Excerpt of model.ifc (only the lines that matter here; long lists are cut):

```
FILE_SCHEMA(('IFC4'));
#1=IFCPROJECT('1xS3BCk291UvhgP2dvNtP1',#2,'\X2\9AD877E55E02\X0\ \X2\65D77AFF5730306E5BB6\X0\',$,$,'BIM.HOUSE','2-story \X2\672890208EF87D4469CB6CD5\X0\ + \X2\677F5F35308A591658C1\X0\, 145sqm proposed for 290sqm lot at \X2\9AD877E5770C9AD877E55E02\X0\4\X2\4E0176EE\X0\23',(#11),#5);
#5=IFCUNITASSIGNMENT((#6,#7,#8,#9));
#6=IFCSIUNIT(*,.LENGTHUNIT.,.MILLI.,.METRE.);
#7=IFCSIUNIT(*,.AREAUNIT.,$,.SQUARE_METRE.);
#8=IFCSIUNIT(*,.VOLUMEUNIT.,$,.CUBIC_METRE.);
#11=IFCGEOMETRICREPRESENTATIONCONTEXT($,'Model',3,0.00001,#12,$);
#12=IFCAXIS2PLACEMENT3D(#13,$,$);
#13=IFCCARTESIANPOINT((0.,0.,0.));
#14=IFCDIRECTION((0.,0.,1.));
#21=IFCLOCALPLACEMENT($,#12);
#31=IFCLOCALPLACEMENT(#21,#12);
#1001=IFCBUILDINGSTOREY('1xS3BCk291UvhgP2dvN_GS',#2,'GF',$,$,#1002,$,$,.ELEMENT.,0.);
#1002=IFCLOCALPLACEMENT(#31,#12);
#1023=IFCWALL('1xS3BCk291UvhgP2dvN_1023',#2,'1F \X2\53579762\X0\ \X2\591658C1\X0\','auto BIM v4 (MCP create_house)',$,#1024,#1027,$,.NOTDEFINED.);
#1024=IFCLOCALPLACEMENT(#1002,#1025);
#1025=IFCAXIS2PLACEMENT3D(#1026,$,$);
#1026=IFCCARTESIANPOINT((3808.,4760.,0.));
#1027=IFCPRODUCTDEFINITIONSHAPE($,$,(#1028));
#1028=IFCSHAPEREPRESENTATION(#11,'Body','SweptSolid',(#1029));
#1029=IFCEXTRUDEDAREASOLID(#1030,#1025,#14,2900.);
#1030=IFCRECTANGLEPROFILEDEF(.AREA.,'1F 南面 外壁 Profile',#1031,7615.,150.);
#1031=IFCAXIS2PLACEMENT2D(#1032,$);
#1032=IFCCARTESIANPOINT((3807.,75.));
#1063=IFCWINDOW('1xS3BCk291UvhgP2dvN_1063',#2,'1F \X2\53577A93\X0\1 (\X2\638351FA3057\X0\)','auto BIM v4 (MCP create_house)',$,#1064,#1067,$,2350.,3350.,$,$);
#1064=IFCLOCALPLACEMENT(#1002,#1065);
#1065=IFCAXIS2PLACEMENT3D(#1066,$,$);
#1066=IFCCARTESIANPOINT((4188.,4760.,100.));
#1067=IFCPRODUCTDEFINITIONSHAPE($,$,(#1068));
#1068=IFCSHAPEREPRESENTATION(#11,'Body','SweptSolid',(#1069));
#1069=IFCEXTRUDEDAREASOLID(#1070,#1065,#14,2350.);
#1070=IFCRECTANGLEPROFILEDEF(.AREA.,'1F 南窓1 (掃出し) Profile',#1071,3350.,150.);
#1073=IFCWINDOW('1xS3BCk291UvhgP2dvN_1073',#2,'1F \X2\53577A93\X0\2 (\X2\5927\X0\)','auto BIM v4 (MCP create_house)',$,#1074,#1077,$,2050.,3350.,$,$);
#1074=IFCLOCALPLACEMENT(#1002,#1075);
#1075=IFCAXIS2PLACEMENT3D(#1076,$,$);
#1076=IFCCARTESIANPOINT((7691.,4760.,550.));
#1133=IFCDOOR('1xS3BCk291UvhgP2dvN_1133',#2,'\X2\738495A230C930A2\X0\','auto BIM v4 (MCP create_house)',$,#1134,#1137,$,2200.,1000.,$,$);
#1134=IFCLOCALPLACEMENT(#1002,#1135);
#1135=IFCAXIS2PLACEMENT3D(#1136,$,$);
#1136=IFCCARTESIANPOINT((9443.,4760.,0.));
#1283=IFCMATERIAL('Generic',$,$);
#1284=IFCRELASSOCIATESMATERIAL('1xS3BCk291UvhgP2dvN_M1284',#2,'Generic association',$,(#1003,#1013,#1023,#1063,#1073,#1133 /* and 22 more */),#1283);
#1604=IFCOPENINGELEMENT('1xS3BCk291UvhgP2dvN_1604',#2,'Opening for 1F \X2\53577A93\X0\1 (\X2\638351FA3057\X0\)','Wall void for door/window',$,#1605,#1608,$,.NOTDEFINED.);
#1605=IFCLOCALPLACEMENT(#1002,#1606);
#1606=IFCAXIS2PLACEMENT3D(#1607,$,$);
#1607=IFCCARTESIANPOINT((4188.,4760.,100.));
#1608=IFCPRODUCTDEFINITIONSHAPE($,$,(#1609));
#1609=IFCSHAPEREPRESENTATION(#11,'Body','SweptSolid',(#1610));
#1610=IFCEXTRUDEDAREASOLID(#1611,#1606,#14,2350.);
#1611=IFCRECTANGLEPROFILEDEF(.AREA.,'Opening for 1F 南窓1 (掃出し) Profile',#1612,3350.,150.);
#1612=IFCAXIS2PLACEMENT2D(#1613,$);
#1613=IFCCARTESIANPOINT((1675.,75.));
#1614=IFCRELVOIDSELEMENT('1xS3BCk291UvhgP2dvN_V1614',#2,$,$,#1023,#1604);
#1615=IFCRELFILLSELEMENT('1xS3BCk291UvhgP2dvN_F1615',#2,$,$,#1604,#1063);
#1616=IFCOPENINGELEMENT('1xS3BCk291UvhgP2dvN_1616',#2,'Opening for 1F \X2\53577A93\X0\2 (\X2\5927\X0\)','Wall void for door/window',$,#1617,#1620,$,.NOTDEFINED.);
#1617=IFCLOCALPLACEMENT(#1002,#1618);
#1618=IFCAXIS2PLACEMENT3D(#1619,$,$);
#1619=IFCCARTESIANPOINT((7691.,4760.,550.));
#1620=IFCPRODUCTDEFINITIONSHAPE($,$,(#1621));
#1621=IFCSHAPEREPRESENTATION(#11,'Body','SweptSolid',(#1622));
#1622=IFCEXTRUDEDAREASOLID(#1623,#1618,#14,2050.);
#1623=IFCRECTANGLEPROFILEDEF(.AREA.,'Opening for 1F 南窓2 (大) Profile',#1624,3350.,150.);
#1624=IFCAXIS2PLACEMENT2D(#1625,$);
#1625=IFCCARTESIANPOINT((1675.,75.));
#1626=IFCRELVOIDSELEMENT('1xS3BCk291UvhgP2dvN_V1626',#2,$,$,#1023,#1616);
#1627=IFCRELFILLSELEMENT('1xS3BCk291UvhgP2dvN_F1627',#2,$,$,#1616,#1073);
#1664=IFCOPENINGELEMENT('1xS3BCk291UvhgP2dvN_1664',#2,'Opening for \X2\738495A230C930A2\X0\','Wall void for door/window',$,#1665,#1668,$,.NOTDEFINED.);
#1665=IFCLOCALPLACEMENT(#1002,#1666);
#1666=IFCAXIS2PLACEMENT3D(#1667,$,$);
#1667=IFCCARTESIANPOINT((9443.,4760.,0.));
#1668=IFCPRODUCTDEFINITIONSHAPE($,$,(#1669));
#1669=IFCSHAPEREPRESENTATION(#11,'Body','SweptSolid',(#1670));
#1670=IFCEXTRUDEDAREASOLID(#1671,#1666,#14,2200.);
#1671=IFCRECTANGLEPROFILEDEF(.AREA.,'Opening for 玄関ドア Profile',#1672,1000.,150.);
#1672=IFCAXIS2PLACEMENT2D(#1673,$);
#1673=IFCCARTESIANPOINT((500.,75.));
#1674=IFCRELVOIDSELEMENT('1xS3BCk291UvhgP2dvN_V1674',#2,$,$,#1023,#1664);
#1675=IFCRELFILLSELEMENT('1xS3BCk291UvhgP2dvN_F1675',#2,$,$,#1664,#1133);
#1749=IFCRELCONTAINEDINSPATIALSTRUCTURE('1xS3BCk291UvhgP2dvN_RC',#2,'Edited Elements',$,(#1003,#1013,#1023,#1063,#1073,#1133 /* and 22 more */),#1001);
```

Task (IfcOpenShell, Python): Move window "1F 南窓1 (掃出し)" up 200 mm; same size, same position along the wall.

```python
import numpy as np
import ifcopenshell
import ifcopenshell.api.geometry
import ifcopenshell.util.placement
import ifcopenshell.util.unit

model = ifcopenshell.open("model.ifc")
unit_scale = ifcopenshell.util.unit.calculate_unit_scale(model)

window = model.by_id(1063)
opening = window.FillsVoids[0].RelatingOpeningElement
dz = 0.2 / unit_scale

shift = np.array([0.0, 0.0, dz])
# The window is not placed relative to its opening, so move both.
for product in (opening, window):
    matrix = ifcopenshell.util.placement.get_local_placement(product.ObjectPlacement)
    matrix[:3, 3] += shift
    ifcopenshell.api.geometry.edit_object_placement(model, product=product, matrix=matrix, is_si=False)

print(f"moved by {dz * unit_scale:+.3f} m")

model.write("model_v2.ifc")
```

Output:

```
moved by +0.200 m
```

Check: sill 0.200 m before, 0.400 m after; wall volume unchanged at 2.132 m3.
